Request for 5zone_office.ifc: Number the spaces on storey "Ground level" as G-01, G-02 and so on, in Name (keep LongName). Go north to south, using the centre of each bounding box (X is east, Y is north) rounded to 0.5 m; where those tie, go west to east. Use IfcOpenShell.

First a look at what the model holds.

```python
import ifcopenshell
import ifcopenshell.util.element
import ifcopenshell.util.placement

model = ifcopenshell.open("5zone_office.ifc")
print(model.schema)
storey = next(s for s in model.by_type("IfcBuildingStorey") if s.Name == "Ground level")
spaces = [e for e in ifcopenshell.util.element.get_decomposition(storey) if e.is_a("IfcSpace")]
for e in sorted(spaces, key=lambda e: e.id()):
    origin = ifcopenshell.util.placement.get_local_placement(e.ObjectPlacement)[:3, 3]
    print(e.id(), e.Name, e.LongName, origin.round(2) + 0.0, sep=" | ")
```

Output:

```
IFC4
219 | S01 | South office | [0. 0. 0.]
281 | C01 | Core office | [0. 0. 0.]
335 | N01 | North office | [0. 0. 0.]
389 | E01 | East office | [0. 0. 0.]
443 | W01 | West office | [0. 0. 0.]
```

```python
import ifcopenshell
import ifcopenshell.geom
import ifcopenshell.util.element
import ifcopenshell.util.shape

model = ifcopenshell.open("5zone_office.ifc")
settings = ifcopenshell.geom.settings()
settings.set("use-world-coords", True)


def centre(element):
    shape = ifcopenshell.geom.create_shape(settings, element)
    return ifcopenshell.util.shape.get_bbox_centroid(shape.geometry)


storey = next(s for s in model.by_type("IfcBuildingStorey") if s.Name == "Ground level")
spaces = [e for e in ifcopenshell.util.element.get_decomposition(storey) if e.is_a("IfcSpace")]

# Insertion points can sit at a corner or the storey origin, so sort by the geometry (in metres).
centres = {e: centre(e) for e in spaces}
spaces.sort(key=lambda e: (-round(centres[e][1] / 0.5), centres[e][0]))

for i, e in enumerate(spaces, start=1):
    number = f"G-{i:02d}"
    e.Name = number
    print(e.id(), number)

model.write("5zone_office_updated.ifc")
```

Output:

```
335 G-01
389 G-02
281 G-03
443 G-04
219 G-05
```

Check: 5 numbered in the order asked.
